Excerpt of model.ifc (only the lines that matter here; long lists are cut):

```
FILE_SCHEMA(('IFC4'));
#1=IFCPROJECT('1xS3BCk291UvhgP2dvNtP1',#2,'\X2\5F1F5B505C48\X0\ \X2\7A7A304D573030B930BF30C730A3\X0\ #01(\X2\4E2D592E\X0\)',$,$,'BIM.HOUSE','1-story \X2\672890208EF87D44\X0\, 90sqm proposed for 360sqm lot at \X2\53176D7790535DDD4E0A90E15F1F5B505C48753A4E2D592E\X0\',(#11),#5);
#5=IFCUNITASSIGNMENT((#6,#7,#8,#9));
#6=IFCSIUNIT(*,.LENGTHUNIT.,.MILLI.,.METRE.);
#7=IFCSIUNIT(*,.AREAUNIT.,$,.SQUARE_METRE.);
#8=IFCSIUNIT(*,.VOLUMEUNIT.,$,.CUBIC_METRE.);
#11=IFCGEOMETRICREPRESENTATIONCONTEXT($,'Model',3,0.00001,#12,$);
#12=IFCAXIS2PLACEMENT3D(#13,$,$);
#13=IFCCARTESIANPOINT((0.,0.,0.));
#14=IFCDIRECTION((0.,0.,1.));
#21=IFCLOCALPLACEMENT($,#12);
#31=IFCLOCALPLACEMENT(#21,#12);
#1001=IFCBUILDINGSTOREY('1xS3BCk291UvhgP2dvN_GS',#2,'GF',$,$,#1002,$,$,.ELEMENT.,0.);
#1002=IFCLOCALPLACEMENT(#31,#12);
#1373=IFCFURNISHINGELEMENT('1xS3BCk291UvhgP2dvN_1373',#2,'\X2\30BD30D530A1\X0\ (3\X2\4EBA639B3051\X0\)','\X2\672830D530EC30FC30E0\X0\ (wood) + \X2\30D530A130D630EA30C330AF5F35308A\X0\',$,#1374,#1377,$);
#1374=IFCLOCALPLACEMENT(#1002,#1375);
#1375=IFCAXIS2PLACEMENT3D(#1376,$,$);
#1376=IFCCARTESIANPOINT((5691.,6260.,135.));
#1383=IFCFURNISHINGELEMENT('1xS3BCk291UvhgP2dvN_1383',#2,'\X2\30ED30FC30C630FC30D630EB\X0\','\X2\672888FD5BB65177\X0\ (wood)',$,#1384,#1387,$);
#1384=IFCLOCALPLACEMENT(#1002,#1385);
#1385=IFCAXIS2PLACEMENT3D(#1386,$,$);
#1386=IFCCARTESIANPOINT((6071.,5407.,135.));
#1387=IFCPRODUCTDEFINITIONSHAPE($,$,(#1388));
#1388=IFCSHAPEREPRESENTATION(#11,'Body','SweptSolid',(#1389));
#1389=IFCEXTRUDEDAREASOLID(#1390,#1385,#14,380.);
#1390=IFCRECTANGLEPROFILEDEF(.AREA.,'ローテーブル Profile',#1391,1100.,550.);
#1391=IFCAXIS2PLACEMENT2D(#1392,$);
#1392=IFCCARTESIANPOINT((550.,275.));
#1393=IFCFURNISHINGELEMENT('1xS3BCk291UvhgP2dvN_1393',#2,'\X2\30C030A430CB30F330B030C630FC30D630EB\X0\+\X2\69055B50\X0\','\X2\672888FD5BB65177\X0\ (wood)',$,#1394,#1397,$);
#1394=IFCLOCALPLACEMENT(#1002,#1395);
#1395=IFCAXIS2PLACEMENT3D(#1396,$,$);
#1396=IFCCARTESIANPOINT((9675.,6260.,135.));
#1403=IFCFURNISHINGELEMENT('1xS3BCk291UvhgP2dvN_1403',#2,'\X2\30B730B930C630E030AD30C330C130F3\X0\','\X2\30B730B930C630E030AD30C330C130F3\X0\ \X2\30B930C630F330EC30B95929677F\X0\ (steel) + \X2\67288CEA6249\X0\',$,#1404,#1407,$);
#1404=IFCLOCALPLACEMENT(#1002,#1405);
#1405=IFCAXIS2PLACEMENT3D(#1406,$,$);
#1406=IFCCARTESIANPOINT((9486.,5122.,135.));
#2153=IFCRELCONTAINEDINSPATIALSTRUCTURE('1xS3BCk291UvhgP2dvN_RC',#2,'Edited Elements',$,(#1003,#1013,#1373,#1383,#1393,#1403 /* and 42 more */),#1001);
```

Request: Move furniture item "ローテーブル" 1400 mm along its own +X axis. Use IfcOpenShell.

```python
import ifcopenshell
import ifcopenshell.api.geometry
import ifcopenshell.util.placement
import ifcopenshell.util.unit

model = ifcopenshell.open("model.ifc")
unit_scale = ifcopenshell.util.unit.calculate_unit_scale(model)

item = model.by_guid("1xS3BCk291UvhgP2dvN_1383")
matrix = ifcopenshell.util.placement.get_local_placement(item.ObjectPlacement)
matrix[:3, 3] += matrix[:3, 0] * 1.4 / unit_scale
ifcopenshell.api.geometry.edit_object_placement(model, product=item, matrix=matrix, is_si=False)

print(ifcopenshell.util.placement.get_local_placement(item.ObjectPlacement).round(3) + 0.0)

model.write("model_rev.ifc")
```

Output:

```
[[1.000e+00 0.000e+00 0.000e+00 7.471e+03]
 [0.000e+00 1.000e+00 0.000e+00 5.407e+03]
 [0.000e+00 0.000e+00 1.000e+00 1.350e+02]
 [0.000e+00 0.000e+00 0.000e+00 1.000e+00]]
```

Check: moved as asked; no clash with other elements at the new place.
